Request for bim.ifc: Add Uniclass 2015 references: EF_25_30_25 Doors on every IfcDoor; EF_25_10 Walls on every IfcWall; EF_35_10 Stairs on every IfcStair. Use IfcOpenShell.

First a look at what the model holds.

```python
import ifcopenshell

model = ifcopenshell.open("bim.ifc")
print(model.schema)
print("classifications:", [c.Name for c in model.by_type("IfcClassification")])
for ifc_class in ("IfcDoor", "IfcRoof", "IfcStair", "IfcWall", "IfcWindow"):
    print(ifc_class, len(model.by_type(ifc_class)))
```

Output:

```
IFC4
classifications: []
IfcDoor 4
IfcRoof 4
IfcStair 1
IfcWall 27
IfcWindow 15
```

```python
import ifcopenshell
import ifcopenshell.api.classification

model = ifcopenshell.open("bim.ifc")

system = ifcopenshell.api.classification.add_classification(model, classification="Uniclass 2015")

codes = {
    "IfcDoor": ("EF_25_30_25", "Doors"),
    "IfcWall": ("EF_25_10", "Walls"),
    "IfcStair": ("EF_35_10", "Stairs"),
}
for ifc_class, (code, name) in codes.items():
    products = model.by_type(ifc_class)
    ifcopenshell.api.classification.add_reference(
        model, products=products, classification=system, identification=code, name=name
    )
    print(code, len(products))

model.write("bim_rev.ifc")
```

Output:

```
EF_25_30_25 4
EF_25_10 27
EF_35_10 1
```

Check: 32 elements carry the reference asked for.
